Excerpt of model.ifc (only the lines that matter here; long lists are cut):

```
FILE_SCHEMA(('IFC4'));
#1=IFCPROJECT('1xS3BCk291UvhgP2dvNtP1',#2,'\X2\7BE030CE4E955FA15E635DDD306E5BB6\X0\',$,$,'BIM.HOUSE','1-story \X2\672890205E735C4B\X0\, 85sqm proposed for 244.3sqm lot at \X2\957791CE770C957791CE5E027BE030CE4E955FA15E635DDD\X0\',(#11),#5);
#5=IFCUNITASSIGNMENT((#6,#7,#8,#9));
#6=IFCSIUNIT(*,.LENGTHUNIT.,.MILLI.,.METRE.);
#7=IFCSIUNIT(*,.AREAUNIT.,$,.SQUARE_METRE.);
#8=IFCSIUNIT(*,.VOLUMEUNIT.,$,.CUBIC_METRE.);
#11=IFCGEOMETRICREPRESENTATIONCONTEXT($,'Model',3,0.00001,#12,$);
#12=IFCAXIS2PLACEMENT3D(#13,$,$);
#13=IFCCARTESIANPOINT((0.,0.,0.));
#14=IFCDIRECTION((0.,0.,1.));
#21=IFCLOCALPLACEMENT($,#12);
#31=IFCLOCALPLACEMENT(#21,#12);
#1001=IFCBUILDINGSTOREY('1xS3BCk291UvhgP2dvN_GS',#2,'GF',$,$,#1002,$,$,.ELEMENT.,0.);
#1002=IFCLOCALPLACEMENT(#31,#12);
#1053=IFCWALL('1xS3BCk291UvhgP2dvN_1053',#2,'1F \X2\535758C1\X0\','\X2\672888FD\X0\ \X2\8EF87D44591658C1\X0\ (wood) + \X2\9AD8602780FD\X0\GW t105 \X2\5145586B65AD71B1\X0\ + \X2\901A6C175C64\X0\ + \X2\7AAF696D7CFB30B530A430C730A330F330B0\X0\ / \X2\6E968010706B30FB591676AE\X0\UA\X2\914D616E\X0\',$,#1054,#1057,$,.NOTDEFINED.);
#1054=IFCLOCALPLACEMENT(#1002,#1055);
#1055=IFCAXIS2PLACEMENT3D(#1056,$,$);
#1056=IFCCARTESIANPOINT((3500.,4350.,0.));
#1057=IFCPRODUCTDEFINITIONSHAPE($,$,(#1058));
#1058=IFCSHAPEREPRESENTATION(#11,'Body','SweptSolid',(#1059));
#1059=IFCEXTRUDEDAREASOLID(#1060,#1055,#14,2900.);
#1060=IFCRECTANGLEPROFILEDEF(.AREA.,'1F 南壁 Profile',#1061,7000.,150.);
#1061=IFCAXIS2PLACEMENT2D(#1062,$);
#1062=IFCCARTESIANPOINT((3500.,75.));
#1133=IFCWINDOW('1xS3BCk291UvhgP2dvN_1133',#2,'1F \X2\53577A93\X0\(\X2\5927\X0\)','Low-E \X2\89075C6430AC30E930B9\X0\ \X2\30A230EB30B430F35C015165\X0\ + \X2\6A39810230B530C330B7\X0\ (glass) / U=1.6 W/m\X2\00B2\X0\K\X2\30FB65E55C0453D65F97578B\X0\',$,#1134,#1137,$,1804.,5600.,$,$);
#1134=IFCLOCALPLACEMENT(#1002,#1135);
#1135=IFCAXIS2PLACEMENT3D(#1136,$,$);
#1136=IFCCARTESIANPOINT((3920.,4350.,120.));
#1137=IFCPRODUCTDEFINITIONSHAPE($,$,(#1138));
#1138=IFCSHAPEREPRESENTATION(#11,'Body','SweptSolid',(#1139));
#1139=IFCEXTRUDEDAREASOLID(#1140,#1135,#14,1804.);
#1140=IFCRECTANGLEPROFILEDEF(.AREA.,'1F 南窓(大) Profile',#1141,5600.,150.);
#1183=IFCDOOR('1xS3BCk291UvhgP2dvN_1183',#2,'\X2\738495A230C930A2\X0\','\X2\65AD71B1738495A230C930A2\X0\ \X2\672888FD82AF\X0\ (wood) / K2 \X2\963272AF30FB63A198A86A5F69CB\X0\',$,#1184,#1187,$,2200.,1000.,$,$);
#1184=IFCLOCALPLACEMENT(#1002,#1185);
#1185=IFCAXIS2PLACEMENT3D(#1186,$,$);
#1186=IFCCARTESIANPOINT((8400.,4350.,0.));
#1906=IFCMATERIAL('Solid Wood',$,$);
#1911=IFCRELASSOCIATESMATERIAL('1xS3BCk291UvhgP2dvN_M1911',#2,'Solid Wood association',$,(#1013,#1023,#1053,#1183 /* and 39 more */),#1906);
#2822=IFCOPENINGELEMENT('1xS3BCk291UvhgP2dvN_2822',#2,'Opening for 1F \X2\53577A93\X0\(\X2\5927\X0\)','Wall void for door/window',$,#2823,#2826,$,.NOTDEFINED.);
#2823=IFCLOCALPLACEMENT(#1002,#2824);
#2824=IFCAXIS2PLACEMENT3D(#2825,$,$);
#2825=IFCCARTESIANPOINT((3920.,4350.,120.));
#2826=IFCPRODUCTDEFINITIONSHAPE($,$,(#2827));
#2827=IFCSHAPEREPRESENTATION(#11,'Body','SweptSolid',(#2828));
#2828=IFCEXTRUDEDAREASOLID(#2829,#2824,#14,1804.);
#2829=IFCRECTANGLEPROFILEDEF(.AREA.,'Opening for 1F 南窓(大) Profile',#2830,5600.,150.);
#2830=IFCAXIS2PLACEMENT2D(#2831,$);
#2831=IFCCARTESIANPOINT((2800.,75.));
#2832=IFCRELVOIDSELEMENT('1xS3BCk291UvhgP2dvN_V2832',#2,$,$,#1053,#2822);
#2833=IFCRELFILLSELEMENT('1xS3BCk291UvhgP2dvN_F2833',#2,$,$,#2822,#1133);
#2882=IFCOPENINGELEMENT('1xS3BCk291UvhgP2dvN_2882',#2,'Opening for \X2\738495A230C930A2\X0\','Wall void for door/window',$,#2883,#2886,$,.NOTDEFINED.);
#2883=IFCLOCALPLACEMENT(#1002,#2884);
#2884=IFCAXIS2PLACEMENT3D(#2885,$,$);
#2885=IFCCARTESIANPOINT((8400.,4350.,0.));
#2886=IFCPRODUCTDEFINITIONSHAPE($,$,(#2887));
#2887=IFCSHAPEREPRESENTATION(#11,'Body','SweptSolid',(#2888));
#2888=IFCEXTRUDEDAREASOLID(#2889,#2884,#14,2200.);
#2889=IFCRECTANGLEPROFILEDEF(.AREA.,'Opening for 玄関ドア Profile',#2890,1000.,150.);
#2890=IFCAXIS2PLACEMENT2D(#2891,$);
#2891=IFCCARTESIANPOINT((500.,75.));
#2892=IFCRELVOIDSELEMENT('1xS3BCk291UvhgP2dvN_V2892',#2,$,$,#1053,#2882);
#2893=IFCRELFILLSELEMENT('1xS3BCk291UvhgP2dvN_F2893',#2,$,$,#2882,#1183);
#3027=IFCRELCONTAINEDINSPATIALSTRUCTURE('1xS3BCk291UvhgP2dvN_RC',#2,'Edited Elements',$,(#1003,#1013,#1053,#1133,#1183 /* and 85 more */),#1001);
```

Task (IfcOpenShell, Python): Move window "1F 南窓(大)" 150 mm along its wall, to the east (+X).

```python
import ifcopenshell
import ifcopenshell.api.geometry
import ifcopenshell.util.placement
import ifcopenshell.util.unit

model = ifcopenshell.open("model.ifc")
unit_scale = ifcopenshell.util.unit.calculate_unit_scale(model)

window = model.by_id(1133)
opening = window.FillsVoids[0].RelatingOpeningElement
wall = opening.VoidsElements[0].RelatingBuildingElement

wall_matrix = ifcopenshell.util.placement.get_local_placement(wall.ObjectPlacement)
shift = wall_matrix[:3, 0] * 0.15 / unit_scale
before = ifcopenshell.util.placement.get_local_placement(window.ObjectPlacement)[:3, 3].copy()

# The window is not placed relative to its opening, so move both.
for product in (opening, window):
    matrix = ifcopenshell.util.placement.get_local_placement(product.ObjectPlacement)
    matrix[:3, 3] += shift
    ifcopenshell.api.geometry.edit_object_placement(model, product=product, matrix=matrix, is_si=False)

after = ifcopenshell.util.placement.get_local_placement(window.ObjectPlacement)[:3, 3]
print("window moved by", (after - before).round(3) + 0.0)

model.write("model_rev.ifc")
```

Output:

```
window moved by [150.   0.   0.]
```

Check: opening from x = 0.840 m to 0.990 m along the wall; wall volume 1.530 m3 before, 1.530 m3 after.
